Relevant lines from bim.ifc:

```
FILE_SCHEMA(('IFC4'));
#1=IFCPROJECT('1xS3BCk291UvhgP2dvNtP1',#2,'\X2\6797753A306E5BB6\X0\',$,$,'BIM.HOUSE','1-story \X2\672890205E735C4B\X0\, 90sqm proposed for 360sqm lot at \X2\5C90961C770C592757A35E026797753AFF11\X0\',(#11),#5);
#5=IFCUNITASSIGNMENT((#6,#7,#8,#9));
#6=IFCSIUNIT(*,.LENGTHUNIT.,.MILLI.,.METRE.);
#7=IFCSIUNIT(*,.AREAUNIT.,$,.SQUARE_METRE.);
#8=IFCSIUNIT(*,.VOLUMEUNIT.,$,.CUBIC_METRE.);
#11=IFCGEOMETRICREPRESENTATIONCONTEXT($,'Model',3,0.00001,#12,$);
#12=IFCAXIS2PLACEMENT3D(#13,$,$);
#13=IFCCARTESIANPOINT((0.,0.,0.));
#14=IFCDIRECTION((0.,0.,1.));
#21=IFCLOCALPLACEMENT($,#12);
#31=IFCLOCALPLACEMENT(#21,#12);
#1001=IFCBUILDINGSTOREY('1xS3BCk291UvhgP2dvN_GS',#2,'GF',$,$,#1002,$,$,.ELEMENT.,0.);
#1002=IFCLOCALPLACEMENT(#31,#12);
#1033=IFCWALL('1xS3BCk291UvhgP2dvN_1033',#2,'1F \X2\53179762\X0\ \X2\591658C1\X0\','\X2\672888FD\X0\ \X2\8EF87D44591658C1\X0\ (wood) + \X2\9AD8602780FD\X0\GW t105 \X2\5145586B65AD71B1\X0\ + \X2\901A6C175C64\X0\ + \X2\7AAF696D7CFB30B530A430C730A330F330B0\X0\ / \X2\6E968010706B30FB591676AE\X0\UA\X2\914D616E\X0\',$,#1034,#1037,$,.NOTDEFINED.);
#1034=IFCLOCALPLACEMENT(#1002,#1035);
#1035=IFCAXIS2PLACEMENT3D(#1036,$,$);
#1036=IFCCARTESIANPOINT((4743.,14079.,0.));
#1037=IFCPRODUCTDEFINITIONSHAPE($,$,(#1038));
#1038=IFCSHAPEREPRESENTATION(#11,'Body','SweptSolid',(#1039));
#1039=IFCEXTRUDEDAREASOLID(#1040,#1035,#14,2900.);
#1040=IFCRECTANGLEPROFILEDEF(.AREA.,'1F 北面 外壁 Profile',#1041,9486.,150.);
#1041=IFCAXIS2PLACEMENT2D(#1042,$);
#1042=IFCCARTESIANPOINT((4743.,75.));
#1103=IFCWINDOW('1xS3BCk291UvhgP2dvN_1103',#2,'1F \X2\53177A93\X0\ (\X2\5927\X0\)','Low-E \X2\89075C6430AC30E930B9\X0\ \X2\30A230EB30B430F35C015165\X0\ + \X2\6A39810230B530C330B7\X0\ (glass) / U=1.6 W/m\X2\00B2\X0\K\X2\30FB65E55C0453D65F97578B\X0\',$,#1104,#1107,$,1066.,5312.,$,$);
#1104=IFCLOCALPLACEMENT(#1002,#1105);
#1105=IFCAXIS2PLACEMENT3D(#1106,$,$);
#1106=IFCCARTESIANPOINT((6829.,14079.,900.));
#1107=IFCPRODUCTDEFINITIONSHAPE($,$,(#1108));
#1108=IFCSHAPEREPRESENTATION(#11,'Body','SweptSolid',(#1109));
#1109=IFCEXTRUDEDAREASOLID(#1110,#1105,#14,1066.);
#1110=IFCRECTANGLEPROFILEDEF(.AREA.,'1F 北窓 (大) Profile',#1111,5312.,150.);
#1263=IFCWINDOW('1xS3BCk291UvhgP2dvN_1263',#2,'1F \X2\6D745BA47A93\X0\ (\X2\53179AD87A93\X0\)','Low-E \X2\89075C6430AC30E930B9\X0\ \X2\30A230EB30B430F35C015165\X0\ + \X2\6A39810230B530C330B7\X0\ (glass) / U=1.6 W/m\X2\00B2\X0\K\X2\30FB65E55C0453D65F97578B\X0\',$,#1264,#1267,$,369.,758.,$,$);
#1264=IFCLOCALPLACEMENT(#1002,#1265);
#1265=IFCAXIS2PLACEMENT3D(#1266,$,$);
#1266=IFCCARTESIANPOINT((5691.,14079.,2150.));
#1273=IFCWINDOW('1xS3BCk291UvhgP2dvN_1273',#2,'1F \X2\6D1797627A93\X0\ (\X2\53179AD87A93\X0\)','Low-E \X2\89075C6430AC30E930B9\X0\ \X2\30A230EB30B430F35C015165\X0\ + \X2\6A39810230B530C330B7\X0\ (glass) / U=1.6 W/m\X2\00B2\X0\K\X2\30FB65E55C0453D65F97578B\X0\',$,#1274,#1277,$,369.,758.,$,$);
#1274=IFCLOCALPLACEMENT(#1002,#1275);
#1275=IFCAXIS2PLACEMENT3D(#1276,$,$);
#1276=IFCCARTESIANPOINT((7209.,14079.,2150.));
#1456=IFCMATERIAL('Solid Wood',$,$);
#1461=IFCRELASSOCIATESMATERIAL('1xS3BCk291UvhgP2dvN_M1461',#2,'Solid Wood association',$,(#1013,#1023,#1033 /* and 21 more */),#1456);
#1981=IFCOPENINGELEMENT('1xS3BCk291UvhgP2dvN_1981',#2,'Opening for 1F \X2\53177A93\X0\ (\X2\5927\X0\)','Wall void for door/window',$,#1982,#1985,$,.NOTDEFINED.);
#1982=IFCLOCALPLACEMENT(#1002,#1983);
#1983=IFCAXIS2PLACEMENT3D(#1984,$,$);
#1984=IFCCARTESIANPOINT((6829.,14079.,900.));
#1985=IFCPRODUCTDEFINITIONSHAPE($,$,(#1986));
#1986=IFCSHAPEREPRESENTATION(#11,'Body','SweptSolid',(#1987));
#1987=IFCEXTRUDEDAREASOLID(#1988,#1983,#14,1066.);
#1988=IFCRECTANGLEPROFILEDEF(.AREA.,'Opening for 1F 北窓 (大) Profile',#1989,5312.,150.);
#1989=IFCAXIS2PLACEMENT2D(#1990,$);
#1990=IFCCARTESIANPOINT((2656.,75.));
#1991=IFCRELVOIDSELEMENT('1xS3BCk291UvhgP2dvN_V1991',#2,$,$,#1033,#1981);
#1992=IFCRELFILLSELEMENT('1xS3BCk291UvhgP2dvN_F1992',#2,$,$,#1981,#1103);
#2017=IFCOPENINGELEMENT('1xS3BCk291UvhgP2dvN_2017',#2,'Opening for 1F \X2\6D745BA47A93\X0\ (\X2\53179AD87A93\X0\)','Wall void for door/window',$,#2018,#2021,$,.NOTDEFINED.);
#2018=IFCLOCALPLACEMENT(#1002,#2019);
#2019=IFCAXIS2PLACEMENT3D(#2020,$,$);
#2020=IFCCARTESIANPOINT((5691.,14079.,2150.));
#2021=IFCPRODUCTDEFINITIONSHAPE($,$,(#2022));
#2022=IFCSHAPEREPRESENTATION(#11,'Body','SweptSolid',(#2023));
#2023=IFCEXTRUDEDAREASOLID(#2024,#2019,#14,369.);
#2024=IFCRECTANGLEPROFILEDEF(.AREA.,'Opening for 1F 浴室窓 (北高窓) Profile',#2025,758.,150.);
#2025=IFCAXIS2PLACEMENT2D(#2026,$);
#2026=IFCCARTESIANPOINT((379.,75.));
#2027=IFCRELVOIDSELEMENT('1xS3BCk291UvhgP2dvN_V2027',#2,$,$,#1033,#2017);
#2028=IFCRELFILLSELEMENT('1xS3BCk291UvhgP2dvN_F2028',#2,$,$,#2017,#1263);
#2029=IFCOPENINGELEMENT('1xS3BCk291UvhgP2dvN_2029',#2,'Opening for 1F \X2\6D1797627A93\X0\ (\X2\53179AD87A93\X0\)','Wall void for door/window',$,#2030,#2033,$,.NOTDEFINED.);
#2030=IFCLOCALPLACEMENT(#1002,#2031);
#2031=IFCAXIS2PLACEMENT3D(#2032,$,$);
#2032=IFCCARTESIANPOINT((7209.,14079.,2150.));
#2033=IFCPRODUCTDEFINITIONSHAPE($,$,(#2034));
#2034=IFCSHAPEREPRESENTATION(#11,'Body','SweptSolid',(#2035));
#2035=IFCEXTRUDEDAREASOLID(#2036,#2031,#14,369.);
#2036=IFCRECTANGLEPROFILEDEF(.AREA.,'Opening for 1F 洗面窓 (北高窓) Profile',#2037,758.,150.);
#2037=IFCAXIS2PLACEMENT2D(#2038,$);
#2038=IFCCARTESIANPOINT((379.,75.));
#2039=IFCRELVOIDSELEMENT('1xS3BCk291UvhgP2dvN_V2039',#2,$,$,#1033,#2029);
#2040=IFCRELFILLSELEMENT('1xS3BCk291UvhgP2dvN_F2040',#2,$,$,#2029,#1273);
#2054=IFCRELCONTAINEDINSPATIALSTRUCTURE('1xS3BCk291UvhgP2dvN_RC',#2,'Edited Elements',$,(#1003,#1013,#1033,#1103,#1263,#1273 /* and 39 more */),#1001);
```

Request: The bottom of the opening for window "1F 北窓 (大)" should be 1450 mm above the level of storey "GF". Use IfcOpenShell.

```python
import numpy as np
import ifcopenshell
import ifcopenshell.api.geometry
import ifcopenshell.geom
import ifcopenshell.util.element
import ifcopenshell.util.placement
import ifcopenshell.util.shape
import ifcopenshell.util.unit

model = ifcopenshell.open("bim.ifc")
unit_scale = ifcopenshell.util.unit.calculate_unit_scale(model)

window = model.by_id(1103)
opening = window.FillsVoids[0].RelatingOpeningElement
storey = ifcopenshell.util.element.get_container(window, ifc_class="IfcBuildingStorey")
level = ifcopenshell.util.placement.get_local_placement(storey.ObjectPlacement)[2, 3]

# The opening's origin need not be at the sill, so measure its lowest point.
shape = ifcopenshell.geom.create_shape(ifcopenshell.geom.settings(), opening)
bottom = ifcopenshell.util.shape.get_shape_bottom_elevation(shape, shape.geometry) / unit_scale
dz = level + 1450.0 - bottom

shift = np.array([0.0, 0.0, dz])
# The window is not placed relative to its opening, so move both.
for product in (opening, window):
    matrix = ifcopenshell.util.placement.get_local_placement(product.ObjectPlacement)
    matrix[:3, 3] += shift
    ifcopenshell.api.geometry.edit_object_placement(model, product=product, matrix=matrix, is_si=False)

print(f"moved by {dz * unit_scale:+.3f} m")

model.write("bim_rev.ifc")
```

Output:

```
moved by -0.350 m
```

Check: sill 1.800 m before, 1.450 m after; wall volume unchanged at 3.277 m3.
